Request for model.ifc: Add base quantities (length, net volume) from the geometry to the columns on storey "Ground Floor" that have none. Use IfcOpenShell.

First a look at what the model holds.

```python
import ifcopenshell
import ifcopenshell.util.element
import ifcopenshell.util.unit

model = ifcopenshell.open("model.ifc")
print(model.schema)
for unit_type in ("LENGTHUNIT", "AREAUNIT", "VOLUMEUNIT"):
    print(unit_type, ifcopenshell.util.unit.calculate_unit_scale(model, unit_type))
storey = next(s for s in model.by_type("IfcBuildingStorey") if s.Name == "Ground Floor")
columns = [e for e in ifcopenshell.util.element.get_decomposition(storey) if e.is_a("IfcColumn")]
for e in sorted(columns, key=lambda e: e.id()):
    print(e.id(), e.is_a(), e.Name, list(ifcopenshell.util.element.get_psets(e, qtos_only=True)), sep=" | ")
```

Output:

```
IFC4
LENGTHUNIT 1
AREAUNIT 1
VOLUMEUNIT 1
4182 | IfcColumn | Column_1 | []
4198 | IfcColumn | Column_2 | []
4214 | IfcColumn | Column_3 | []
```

```python
import ifcopenshell
import ifcopenshell.api.pset
import ifcopenshell.geom
import ifcopenshell.util.element
import ifcopenshell.util.shape
import ifcopenshell.util.unit

model = ifcopenshell.open("model.ifc")
unit_scale = ifcopenshell.util.unit.calculate_unit_scale(model)
volume_scale = ifcopenshell.util.unit.calculate_unit_scale(model, "VOLUMEUNIT")
settings = ifcopenshell.geom.settings()

storey = next(s for s in model.by_type("IfcBuildingStorey") if s.Name == "Ground Floor")
columns = [e for e in ifcopenshell.util.element.get_decomposition(storey) if e.is_a("IfcColumn")]

for e in sorted(columns, key=lambda e: e.id()):
    if ifcopenshell.util.element.get_psets(e, qtos_only=True, should_inherit=False):
        continue
    # Geometry comes back in metres, in the element's own axes.
    shape = ifcopenshell.geom.create_shape(settings, e)
    values = {
        "Length": ifcopenshell.util.shape.get_z(shape.geometry) / unit_scale,
        "NetVolume": ifcopenshell.util.shape.get_volume(shape.geometry) / volume_scale,
    }
    qto = ifcopenshell.api.pset.add_qto(model, product=e, name="Qto_ColumnBaseQuantities")
    ifcopenshell.api.pset.edit_qto(model, qto=qto, properties=values)
    print(e.id(), {k: round(v, 3) for k, v in values.items()})

model.write("model-out.ifc")
```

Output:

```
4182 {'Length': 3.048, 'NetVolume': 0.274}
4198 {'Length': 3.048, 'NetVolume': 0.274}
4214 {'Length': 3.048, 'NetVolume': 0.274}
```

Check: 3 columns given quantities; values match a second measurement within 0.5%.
